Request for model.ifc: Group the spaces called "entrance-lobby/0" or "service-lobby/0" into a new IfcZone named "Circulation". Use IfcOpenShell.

First a look at what the model holds.

```python
import ifcopenshell

model = ifcopenshell.open("model.ifc")
print(model.schema)
seen = {}
for space in model.by_type("IfcSpace"):
    seen[space.Name] = seen.get(space.Name, 0) + 1
for name, count in sorted(seen.items(), key=str):
    print(count, "x", name)
print("zones:", [z.Name for z in model.by_type("IfcZone")][:20])
```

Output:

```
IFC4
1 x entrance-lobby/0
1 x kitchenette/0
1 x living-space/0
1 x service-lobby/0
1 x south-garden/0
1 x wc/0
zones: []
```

```python
import ifcopenshell
import ifcopenshell.api.group
import ifcopenshell.api.root

model = ifcopenshell.open("model.ifc")

names = {"entrance-lobby/0", "service-lobby/0"}
spaces = [s for s in model.by_type("IfcSpace") if s.Name in names]

zone = ifcopenshell.api.root.create_entity(model, ifc_class="IfcZone", name="Circulation")
ifcopenshell.api.group.assign_group(model, products=spaces, group=zone)
print(len(spaces), "spaces in", zone.Name)

model.write("model-out.ifc")
```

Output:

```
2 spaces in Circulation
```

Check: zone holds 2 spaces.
